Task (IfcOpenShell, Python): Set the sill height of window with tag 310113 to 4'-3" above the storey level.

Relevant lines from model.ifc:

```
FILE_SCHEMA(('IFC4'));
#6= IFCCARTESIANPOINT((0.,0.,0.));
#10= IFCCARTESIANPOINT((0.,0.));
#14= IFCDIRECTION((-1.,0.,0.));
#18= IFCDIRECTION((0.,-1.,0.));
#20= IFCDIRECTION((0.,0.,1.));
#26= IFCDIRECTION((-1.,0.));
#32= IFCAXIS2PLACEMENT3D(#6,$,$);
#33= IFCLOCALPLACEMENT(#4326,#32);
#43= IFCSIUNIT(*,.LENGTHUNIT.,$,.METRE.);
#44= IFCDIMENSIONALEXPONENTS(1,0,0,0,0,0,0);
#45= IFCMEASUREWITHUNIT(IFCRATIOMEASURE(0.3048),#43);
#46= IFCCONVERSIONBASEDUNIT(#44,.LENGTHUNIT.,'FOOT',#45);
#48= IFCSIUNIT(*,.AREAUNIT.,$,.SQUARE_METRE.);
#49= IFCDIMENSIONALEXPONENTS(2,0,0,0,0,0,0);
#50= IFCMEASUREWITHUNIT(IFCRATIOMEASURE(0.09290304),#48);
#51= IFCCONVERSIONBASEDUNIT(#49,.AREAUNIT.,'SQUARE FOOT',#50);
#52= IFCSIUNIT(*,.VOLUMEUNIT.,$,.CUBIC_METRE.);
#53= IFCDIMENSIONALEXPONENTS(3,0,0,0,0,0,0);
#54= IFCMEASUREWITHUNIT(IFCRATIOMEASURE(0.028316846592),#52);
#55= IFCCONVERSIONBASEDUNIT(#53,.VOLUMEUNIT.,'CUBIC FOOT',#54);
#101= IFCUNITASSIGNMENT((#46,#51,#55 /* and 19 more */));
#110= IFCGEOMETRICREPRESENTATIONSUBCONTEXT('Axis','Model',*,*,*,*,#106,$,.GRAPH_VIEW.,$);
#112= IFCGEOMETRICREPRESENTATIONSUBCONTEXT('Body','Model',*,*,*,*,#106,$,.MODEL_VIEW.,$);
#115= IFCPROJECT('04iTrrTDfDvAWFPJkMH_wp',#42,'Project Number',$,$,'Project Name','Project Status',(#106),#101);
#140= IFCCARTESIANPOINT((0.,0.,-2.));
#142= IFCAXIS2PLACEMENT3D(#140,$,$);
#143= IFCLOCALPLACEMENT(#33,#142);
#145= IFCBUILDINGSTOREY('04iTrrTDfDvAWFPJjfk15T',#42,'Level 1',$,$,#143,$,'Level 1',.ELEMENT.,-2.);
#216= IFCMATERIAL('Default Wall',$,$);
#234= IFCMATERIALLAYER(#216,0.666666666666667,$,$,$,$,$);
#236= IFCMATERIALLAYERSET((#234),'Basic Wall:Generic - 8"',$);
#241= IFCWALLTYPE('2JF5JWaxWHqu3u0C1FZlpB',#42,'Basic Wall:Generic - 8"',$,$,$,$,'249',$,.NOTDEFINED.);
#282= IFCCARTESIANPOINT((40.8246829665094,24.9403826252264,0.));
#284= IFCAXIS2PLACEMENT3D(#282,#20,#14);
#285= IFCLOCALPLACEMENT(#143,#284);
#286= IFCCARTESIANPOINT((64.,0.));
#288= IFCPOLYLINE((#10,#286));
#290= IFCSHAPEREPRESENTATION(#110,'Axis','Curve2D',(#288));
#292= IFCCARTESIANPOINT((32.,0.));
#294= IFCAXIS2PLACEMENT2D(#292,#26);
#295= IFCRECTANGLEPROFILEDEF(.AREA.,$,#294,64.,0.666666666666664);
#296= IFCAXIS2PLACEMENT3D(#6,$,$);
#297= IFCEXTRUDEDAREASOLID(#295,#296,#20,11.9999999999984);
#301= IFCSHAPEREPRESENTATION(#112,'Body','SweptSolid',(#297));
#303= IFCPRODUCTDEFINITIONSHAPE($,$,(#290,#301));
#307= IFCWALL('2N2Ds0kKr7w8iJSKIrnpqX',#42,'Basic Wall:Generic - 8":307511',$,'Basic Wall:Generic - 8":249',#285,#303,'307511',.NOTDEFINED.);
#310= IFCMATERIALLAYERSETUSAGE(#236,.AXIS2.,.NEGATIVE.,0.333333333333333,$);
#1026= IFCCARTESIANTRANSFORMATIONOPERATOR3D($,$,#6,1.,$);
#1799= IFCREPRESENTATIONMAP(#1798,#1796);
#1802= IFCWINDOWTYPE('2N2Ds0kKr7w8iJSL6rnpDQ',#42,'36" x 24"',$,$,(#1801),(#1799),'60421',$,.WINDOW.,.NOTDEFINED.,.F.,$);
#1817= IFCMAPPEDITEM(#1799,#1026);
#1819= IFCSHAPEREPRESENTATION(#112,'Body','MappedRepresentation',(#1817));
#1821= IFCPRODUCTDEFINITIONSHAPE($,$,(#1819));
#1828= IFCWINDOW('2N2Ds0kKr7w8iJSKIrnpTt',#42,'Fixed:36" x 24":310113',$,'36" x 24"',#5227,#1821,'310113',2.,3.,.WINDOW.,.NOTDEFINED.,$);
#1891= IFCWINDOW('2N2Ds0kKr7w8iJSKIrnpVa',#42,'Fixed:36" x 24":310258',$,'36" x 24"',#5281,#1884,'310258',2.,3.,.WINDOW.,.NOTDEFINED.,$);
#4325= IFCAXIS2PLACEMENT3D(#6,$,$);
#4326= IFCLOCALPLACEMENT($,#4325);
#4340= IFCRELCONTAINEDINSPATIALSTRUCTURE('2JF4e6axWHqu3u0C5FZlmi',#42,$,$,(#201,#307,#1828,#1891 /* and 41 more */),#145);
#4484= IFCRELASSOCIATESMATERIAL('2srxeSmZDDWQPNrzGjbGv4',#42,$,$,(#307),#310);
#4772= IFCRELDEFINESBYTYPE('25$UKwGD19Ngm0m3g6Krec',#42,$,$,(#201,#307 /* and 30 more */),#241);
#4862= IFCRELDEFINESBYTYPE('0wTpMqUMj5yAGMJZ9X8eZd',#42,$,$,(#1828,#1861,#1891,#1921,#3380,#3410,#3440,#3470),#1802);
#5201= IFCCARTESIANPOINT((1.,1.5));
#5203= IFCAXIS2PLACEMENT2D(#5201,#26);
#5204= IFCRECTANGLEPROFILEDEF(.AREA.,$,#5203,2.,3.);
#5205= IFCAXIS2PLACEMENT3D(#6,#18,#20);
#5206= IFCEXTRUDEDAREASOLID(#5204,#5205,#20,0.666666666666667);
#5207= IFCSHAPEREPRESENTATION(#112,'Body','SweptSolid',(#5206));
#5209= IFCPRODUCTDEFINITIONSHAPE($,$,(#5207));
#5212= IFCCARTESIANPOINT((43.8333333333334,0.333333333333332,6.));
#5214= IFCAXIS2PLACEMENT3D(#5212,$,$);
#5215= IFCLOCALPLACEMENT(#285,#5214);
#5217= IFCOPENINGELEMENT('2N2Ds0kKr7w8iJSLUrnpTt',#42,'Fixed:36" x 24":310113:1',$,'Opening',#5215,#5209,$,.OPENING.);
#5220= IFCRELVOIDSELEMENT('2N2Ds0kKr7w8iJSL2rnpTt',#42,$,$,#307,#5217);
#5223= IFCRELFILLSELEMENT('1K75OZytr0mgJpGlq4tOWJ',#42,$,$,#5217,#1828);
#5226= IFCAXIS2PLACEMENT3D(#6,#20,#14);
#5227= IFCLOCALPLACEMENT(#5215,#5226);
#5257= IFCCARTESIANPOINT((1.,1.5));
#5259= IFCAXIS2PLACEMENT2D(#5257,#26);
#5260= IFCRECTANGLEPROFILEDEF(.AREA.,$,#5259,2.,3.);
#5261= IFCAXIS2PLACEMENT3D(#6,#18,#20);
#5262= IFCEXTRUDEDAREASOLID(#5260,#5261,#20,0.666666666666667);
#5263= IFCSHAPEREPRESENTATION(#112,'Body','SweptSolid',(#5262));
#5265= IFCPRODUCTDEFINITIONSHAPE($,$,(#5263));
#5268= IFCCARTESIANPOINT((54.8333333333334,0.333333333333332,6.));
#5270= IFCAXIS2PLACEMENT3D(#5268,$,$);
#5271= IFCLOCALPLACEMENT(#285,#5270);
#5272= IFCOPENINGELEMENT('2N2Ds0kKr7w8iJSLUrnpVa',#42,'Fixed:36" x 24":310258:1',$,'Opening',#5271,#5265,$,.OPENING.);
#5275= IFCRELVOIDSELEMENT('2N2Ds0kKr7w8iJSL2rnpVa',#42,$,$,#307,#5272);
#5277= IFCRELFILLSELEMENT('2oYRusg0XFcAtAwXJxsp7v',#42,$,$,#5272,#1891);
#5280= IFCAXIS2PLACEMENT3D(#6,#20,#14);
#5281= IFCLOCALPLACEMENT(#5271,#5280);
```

```python
import numpy as np
import ifcopenshell
import ifcopenshell.api.geometry
import ifcopenshell.geom
import ifcopenshell.util.element
import ifcopenshell.util.placement
import ifcopenshell.util.shape
import ifcopenshell.util.unit

model = ifcopenshell.open("model.ifc")
unit_scale = ifcopenshell.util.unit.calculate_unit_scale(model)

window = model.by_id(1828)
opening = window.FillsVoids[0].RelatingOpeningElement
storey = ifcopenshell.util.element.get_container(window, ifc_class="IfcBuildingStorey")
level = ifcopenshell.util.placement.get_local_placement(storey.ObjectPlacement)[2, 3]

# The opening's origin need not be at the sill, so measure its lowest point.
shape = ifcopenshell.geom.create_shape(ifcopenshell.geom.settings(), opening)
bottom = ifcopenshell.util.shape.get_shape_bottom_elevation(shape, shape.geometry) / unit_scale
dz = level + 51 * 0.0254 / unit_scale - bottom

shift = np.array([0.0, 0.0, dz])
# The window is placed relative to its opening, so it follows when the opening moves.
matrix = ifcopenshell.util.placement.get_local_placement(opening.ObjectPlacement)
matrix[:3, 3] += shift
ifcopenshell.api.geometry.edit_object_placement(
    model, product=opening, matrix=matrix, is_si=False, should_transform_children=True
)

print(f"moved by {dz * unit_scale:+.3f} m")

model.write("model_updated.ifc")
```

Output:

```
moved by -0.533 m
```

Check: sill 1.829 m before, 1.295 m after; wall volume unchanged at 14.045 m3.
